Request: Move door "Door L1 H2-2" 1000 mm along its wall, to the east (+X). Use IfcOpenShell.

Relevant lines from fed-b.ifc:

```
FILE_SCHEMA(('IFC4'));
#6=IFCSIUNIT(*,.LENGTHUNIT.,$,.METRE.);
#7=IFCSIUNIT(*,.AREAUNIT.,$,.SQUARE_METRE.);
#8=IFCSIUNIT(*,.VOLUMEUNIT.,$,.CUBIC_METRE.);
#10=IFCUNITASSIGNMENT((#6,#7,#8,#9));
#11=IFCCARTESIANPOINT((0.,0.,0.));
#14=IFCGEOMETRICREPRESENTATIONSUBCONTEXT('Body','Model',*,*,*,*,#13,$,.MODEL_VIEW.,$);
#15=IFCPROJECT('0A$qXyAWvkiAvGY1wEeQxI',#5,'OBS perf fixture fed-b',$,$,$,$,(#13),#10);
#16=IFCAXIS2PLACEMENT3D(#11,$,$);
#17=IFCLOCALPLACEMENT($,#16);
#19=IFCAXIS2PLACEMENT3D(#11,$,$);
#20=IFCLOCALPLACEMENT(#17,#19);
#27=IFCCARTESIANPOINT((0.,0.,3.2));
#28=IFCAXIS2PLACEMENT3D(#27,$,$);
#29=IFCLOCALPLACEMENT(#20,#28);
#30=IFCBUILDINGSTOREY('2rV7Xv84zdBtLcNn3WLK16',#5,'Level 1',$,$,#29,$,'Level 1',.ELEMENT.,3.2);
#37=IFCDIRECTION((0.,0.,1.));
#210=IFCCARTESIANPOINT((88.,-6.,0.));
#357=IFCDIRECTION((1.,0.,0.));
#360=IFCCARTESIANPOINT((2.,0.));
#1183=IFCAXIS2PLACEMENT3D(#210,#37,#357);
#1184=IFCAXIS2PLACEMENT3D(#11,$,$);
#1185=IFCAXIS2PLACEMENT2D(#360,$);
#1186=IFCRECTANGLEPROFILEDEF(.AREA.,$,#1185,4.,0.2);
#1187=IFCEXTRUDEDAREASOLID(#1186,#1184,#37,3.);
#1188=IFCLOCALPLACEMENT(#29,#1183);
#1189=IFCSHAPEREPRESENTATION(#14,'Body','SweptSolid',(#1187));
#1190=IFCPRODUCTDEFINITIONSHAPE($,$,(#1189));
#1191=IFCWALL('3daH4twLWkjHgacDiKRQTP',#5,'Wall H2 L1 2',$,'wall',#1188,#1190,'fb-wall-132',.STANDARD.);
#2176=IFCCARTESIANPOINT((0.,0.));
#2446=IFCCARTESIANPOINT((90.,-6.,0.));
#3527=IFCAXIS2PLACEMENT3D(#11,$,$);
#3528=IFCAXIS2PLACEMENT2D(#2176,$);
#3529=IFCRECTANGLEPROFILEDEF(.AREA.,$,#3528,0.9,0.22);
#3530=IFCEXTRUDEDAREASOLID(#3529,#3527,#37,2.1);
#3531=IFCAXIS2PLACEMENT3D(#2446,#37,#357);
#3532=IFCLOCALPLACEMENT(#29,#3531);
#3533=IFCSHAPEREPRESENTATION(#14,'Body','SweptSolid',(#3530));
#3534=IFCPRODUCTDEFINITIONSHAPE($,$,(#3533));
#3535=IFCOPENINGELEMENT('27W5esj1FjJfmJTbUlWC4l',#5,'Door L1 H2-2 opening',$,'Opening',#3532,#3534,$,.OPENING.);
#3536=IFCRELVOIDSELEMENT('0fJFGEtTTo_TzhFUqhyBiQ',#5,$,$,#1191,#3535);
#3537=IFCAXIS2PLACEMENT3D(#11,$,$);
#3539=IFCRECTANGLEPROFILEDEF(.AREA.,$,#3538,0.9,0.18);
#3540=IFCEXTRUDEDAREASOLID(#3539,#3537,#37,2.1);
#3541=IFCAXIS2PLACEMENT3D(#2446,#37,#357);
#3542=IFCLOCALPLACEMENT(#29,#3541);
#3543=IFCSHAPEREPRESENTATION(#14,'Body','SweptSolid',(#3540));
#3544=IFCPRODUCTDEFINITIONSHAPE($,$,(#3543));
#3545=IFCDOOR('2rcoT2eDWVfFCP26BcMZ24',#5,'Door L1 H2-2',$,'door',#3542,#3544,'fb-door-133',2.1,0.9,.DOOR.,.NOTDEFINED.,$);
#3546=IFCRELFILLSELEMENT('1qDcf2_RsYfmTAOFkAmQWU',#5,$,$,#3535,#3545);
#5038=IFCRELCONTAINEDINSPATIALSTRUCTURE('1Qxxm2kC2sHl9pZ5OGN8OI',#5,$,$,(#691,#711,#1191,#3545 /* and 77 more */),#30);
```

```python
import ifcopenshell
import ifcopenshell.api.geometry
import ifcopenshell.util.placement
import ifcopenshell.util.unit

model = ifcopenshell.open("fed-b.ifc")
unit_scale = ifcopenshell.util.unit.calculate_unit_scale(model)

door = model.by_guid("2rcoT2eDWVfFCP26BcMZ24")
opening = door.FillsVoids[0].RelatingOpeningElement
wall = opening.VoidsElements[0].RelatingBuildingElement

wall_matrix = ifcopenshell.util.placement.get_local_placement(wall.ObjectPlacement)
shift = wall_matrix[:3, 0] * 1 / unit_scale
before = ifcopenshell.util.placement.get_local_placement(door.ObjectPlacement)[:3, 3].copy()

# The door is not placed relative to its opening, so move both.
for product in (opening, door):
    matrix = ifcopenshell.util.placement.get_local_placement(product.ObjectPlacement)
    matrix[:3, 3] += shift
    ifcopenshell.api.geometry.edit_object_placement(model, product=product, matrix=matrix, is_si=False)

after = ifcopenshell.util.placement.get_local_placement(door.ObjectPlacement)[:3, 3]
print("door moved by", (after - before).round(3) + 0.0)

model.write("fed-b_updated.ifc")
```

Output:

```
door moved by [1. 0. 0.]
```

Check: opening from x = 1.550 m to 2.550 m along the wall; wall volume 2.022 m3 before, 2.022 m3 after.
